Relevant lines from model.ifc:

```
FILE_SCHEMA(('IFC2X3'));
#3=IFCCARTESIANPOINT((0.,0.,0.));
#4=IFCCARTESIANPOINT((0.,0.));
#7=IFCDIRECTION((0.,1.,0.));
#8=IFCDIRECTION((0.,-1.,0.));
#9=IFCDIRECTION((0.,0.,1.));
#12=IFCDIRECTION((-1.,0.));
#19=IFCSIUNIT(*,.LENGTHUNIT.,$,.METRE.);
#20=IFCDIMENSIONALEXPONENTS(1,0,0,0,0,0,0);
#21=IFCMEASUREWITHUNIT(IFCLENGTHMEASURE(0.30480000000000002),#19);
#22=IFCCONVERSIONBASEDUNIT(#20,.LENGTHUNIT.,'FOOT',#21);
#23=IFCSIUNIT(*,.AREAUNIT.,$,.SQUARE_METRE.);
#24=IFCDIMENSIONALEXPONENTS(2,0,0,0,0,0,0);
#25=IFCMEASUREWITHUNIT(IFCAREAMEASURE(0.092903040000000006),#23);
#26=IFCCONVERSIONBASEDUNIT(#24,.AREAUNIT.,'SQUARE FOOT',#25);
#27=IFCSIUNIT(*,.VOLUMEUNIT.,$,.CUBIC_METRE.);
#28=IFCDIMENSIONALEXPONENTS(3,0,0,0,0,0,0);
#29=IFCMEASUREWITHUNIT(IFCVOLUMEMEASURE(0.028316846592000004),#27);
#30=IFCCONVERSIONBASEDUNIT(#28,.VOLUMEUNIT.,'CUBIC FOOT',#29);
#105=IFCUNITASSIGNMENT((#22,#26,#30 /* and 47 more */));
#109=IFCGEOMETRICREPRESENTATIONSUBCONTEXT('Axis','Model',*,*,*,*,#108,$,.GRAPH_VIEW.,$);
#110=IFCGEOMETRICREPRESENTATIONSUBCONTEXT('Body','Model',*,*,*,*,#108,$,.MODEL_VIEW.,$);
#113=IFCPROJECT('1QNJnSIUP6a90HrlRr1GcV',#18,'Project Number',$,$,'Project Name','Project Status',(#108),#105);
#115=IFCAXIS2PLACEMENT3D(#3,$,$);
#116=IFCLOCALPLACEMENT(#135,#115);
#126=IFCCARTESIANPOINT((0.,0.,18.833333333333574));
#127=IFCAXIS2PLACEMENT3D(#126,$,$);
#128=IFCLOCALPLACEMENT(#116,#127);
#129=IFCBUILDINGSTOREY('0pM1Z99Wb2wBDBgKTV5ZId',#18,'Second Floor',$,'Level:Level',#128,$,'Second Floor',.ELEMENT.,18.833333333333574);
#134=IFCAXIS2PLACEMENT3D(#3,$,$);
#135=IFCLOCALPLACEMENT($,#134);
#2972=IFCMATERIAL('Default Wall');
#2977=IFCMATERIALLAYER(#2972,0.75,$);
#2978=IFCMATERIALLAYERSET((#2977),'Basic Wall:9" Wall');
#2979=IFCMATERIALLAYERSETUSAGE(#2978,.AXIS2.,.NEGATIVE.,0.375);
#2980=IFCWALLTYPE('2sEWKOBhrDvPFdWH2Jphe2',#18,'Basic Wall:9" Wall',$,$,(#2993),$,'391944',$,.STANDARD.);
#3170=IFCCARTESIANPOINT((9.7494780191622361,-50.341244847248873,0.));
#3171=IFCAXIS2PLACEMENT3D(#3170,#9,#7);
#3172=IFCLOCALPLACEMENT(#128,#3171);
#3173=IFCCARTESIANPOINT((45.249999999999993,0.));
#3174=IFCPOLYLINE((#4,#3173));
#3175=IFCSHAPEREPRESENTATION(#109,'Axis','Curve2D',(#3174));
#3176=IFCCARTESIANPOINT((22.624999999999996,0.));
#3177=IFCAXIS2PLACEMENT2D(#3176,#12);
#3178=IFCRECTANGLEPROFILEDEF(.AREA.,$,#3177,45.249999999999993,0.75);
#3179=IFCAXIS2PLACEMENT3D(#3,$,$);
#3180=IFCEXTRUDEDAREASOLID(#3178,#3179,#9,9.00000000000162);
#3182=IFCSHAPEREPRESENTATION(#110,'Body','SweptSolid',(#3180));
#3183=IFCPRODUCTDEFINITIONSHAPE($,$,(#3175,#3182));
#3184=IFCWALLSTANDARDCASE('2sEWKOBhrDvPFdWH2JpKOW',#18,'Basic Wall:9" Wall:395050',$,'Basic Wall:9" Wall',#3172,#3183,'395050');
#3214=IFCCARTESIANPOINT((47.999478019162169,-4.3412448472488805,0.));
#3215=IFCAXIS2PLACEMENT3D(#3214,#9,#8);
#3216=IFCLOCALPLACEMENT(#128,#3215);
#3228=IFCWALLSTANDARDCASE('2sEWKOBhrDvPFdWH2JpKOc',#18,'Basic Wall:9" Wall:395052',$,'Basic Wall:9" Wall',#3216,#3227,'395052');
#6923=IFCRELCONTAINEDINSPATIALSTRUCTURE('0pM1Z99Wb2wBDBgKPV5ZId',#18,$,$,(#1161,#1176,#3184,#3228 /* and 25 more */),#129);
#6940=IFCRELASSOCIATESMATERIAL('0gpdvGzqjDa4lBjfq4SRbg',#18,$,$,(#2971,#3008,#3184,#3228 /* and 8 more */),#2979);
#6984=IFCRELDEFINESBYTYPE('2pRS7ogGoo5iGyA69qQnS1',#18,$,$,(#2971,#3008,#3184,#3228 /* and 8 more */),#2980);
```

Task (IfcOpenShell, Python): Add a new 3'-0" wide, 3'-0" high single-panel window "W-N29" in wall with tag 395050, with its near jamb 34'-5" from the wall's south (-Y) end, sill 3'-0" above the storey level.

```python
import numpy as np
import ifcopenshell
import ifcopenshell.api.feature
import ifcopenshell.api.geometry
import ifcopenshell.api.root
import ifcopenshell.api.spatial
import ifcopenshell.api.type
import ifcopenshell.geom
import ifcopenshell.util.element
import ifcopenshell.util.placement
import ifcopenshell.util.representation
import ifcopenshell.util.shape
import ifcopenshell.util.unit

model = ifcopenshell.open("model.ifc")
unit_scale = ifcopenshell.util.unit.calculate_unit_scale(model)
settings = ifcopenshell.geom.settings()


def volume(element):
    """Net volume in cubic metres, openings subtracted."""
    shape = ifcopenshell.geom.create_shape(settings, element)
    return ifcopenshell.util.shape.get_volume(shape.geometry)


wall = model.by_guid("2sEWKOBhrDvPFdWH2JpKOW")
storey = ifcopenshell.util.element.get_container(wall, ifc_class="IfcBuildingStorey")
context = ifcopenshell.util.representation.get_context(model, "Model", "Body", "MODEL_VIEW")
before = volume(wall)

width, height, from_end, sill = 0.9144, 0.9144, 10.4902, 0.9144  # metres

# The wall runs along its own X axis, and the end named is its -X end.
wall_shape = ifcopenshell.geom.create_shape(settings, wall)
x, y, z = ifcopenshell.util.shape.get_vertices(wall_shape.geometry).T
start = x.min() + from_end
face, thickness = float(y.min()), float(y.max() - y.min())
wall_matrix = ifcopenshell.util.placement.get_local_placement(wall.ObjectPlacement)
level = ifcopenshell.util.placement.get_local_placement(storey.ObjectPlacement)[2, 3]


def in_wall(x, y):
    """Placement at x, y metres in the wall's axes, at sill height."""
    matrix = wall_matrix.copy()
    matrix[:, 3] = wall_matrix @ np.array([x / unit_scale, y / unit_scale, 0.0, 1.0])
    matrix[2, 3] = level + sill / unit_scale
    return matrix


# Opening: a box that overshoots both wall faces by 50 mm.
opening = ifcopenshell.api.root.create_entity(model, ifc_class="IfcOpeningElement")
box = ifcopenshell.api.geometry.add_wall_representation(
    model, context=context, length=width, height=height, thickness=thickness + 0.1
)
ifcopenshell.api.geometry.assign_representation(model, product=opening, representation=box)
ifcopenshell.api.geometry.edit_object_placement(model, product=opening, matrix=in_wall(start, face - 0.05), is_si=False)
ifcopenshell.api.feature.add_feature(model, feature=opening, element=wall)

window = ifcopenshell.api.root.create_entity(model, ifc_class="IfcWindow", name="W-N29")
window.OverallWidth, window.OverallHeight = width / unit_scale, height / unit_scale
body = ifcopenshell.api.geometry.add_window_representation(
    model,
    context=context,
    overall_width=window.OverallWidth,
    overall_height=window.OverallHeight,
    partition_type="SINGLE_PANEL",
)
ifcopenshell.api.geometry.assign_representation(model, product=window, representation=body)
ifcopenshell.api.spatial.assign_container(model, products=[window], relating_structure=storey)
fills = ifcopenshell.api.feature.add_filling(model, opening=opening, element=window)
fills.OwnerHistory = window.OwnerHistory  # required in IFC2X3

# IFC2X3 keeps the operation on the window style.
style = ifcopenshell.api.root.create_entity(model, ifc_class="IfcWindowStyle", name="W-N29")
style.OperationType, style.ConstructionType = "SINGLE_PANEL", "NOTDEFINED"
style.ParameterTakesPrecedence = style.Sizeable = False
ifcopenshell.api.type.assign_type(model, related_objects=[window], relating_type=style)

# Centre the window in the wall's thickness.
ifcopenshell.api.geometry.edit_object_placement(model, product=window, matrix=in_wall(start, face), is_si=False)
window_shape = ifcopenshell.geom.create_shape(settings, window)
depth = ifcopenshell.util.shape.get_vertices(window_shape.geometry)[:, 1]
offset = face + thickness / 2 - (depth.min() + depth.max()) / 2
ifcopenshell.api.geometry.edit_object_placement(model, product=window, matrix=in_wall(start, offset), is_si=False)

after = volume(wall)

print(f"wall volume {before:.3f} -> {after:.3f} m3")

model.write("model-out.ifc")
```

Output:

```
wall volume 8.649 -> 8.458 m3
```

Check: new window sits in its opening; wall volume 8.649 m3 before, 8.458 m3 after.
